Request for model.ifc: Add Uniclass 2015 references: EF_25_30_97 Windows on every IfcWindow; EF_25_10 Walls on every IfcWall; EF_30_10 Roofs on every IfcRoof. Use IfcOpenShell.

First a look at what the model holds.

```python
import ifcopenshell

model = ifcopenshell.open("model.ifc")
print(model.schema)
print("classifications:", [c.Name for c in model.by_type("IfcClassification")])
for ifc_class in ("IfcDoor", "IfcRoof", "IfcStair", "IfcWall", "IfcWindow"):
    print(ifc_class, len(model.by_type(ifc_class)))
```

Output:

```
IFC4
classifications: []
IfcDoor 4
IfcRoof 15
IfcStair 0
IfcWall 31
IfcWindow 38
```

```python
import ifcopenshell
import ifcopenshell.api.classification

model = ifcopenshell.open("model.ifc")

system = ifcopenshell.api.classification.add_classification(model, classification="Uniclass 2015")

codes = {
    "IfcWindow": ("EF_25_30_97", "Windows"),
    "IfcWall": ("EF_25_10", "Walls"),
    "IfcRoof": ("EF_30_10", "Roofs"),
}
for ifc_class, (code, name) in codes.items():
    products = model.by_type(ifc_class)
    ifcopenshell.api.classification.add_reference(
        model, products=products, classification=system, identification=code, name=name
    )
    print(code, len(products))

model.write("model_edited.ifc")
```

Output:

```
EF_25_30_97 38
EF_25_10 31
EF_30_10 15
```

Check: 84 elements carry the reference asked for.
